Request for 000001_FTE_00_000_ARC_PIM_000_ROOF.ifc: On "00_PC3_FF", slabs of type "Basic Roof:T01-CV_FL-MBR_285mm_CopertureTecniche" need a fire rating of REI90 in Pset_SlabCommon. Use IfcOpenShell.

First a look at what the model holds.

```python
import ifcopenshell
import ifcopenshell.util.element

model = ifcopenshell.open("000001_FTE_00_000_ARC_PIM_000_ROOF.ifc")
print(model.schema)
storey = next(s for s in model.by_type("IfcBuildingStorey") if s.Name == "00_PC3_FF")
slabs = [e for e in ifcopenshell.util.element.get_decomposition(storey) if e.is_a("IfcSlab")]
seen = {}
for e in slabs:
    element_type = ifcopenshell.util.element.get_type(e)
    key = (element_type.Name if element_type != e and element_type else None, ifcopenshell.util.element.get_pset(e, "Pset_SlabCommon", "FireRating"))
    seen[key] = seen.get(key, 0) + 1
for (name, value), count in sorted(seen.items(), key=str):
    print(count, "x", name, "|", value)
```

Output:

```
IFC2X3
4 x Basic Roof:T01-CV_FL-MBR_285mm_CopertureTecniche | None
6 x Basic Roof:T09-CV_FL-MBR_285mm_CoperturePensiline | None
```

```python
import ifcopenshell
import ifcopenshell.api.pset
import ifcopenshell.util.element

model = ifcopenshell.open("000001_FTE_00_000_ARC_PIM_000_ROOF.ifc")

storey = next(s for s in model.by_type("IfcBuildingStorey") if s.Name == "00_PC3_FF")
slabs = [e for e in ifcopenshell.util.element.get_decomposition(storey) if e.is_a("IfcSlab")]

count = 0
for e in slabs:
    element_type = ifcopenshell.util.element.get_type(e)
    if element_type in (None, e) or element_type.Name != "Basic Roof:T01-CV_FL-MBR_285mm_CopertureTecniche":
        continue
    # add_pset returns the element's existing set when there is one.
    pset = ifcopenshell.api.pset.add_pset(model, product=e, name="Pset_SlabCommon")
    ifcopenshell.api.pset.edit_pset(model, pset=pset, properties={"FireRating": "REI90"})
    count += 1

print(count, "slabs updated")

model.write("000001_FTE_00_000_ARC_PIM_000_ROOF_edited.ifc")
```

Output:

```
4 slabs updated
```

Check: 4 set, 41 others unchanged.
